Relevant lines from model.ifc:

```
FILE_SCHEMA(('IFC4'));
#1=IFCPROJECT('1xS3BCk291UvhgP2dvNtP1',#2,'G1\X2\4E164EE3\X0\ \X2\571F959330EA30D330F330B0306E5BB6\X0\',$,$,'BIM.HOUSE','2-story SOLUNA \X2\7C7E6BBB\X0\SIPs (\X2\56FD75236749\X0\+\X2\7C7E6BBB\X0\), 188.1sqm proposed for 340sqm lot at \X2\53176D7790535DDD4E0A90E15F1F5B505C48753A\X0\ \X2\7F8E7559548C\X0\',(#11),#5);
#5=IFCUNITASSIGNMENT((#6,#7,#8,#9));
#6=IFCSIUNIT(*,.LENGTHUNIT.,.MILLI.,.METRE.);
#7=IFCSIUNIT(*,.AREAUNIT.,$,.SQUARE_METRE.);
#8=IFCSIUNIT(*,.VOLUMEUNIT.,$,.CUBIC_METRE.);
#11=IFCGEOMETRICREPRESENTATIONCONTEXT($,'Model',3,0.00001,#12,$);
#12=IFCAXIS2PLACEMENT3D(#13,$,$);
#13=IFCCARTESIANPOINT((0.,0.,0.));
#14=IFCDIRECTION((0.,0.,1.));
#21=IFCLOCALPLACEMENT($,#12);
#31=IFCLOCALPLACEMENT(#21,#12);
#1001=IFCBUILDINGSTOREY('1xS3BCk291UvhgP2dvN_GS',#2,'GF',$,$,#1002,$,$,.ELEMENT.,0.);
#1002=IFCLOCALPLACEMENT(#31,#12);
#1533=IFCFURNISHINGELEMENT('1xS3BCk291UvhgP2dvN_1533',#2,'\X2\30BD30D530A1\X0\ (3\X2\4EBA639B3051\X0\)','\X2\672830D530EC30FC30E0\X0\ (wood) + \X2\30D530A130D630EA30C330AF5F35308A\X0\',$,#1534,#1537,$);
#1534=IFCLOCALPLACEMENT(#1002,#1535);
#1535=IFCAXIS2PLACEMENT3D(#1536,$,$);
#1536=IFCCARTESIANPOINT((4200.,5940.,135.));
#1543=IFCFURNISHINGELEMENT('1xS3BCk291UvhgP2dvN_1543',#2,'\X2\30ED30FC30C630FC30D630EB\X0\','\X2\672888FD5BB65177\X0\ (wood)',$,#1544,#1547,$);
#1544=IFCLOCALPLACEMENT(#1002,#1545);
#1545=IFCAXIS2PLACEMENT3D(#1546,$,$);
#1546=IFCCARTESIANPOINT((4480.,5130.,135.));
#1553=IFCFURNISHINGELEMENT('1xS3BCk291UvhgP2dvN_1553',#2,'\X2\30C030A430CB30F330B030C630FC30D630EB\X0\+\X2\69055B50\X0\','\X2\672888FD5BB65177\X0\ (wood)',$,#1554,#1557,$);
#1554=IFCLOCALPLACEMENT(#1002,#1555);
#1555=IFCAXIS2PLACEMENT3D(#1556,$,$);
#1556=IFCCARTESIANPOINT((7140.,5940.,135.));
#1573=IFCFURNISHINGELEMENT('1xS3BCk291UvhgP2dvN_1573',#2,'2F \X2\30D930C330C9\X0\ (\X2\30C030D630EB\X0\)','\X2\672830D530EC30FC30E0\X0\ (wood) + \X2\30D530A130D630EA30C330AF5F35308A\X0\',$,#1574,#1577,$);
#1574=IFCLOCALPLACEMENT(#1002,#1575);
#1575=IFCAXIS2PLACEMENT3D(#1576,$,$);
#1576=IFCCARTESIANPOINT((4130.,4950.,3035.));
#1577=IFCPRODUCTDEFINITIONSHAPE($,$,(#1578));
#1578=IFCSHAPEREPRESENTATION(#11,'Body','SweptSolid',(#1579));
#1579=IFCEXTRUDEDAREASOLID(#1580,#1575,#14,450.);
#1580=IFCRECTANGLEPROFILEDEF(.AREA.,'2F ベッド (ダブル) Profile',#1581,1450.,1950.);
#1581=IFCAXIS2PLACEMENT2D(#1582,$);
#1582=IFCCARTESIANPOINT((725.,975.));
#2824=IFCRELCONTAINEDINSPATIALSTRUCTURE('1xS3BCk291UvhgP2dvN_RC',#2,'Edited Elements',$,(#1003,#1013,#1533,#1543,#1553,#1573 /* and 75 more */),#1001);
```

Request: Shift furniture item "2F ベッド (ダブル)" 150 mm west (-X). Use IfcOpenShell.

```python
import ifcopenshell
import ifcopenshell.api.geometry
import ifcopenshell.util.placement

model = ifcopenshell.open("model.ifc")

item = model.by_guid("1xS3BCk291UvhgP2dvN_1573")
matrix = ifcopenshell.util.placement.get_local_placement(item.ObjectPlacement)
matrix[0, 3] -= 150.0
ifcopenshell.api.geometry.edit_object_placement(model, product=item, matrix=matrix, is_si=False)

print(ifcopenshell.util.placement.get_local_placement(item.ObjectPlacement).round(3) + 0.0)

model.write("model-out.ifc")
```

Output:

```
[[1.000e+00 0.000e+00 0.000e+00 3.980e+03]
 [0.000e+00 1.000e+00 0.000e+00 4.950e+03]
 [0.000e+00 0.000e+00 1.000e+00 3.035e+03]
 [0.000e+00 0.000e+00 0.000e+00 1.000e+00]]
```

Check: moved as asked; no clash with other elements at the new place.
